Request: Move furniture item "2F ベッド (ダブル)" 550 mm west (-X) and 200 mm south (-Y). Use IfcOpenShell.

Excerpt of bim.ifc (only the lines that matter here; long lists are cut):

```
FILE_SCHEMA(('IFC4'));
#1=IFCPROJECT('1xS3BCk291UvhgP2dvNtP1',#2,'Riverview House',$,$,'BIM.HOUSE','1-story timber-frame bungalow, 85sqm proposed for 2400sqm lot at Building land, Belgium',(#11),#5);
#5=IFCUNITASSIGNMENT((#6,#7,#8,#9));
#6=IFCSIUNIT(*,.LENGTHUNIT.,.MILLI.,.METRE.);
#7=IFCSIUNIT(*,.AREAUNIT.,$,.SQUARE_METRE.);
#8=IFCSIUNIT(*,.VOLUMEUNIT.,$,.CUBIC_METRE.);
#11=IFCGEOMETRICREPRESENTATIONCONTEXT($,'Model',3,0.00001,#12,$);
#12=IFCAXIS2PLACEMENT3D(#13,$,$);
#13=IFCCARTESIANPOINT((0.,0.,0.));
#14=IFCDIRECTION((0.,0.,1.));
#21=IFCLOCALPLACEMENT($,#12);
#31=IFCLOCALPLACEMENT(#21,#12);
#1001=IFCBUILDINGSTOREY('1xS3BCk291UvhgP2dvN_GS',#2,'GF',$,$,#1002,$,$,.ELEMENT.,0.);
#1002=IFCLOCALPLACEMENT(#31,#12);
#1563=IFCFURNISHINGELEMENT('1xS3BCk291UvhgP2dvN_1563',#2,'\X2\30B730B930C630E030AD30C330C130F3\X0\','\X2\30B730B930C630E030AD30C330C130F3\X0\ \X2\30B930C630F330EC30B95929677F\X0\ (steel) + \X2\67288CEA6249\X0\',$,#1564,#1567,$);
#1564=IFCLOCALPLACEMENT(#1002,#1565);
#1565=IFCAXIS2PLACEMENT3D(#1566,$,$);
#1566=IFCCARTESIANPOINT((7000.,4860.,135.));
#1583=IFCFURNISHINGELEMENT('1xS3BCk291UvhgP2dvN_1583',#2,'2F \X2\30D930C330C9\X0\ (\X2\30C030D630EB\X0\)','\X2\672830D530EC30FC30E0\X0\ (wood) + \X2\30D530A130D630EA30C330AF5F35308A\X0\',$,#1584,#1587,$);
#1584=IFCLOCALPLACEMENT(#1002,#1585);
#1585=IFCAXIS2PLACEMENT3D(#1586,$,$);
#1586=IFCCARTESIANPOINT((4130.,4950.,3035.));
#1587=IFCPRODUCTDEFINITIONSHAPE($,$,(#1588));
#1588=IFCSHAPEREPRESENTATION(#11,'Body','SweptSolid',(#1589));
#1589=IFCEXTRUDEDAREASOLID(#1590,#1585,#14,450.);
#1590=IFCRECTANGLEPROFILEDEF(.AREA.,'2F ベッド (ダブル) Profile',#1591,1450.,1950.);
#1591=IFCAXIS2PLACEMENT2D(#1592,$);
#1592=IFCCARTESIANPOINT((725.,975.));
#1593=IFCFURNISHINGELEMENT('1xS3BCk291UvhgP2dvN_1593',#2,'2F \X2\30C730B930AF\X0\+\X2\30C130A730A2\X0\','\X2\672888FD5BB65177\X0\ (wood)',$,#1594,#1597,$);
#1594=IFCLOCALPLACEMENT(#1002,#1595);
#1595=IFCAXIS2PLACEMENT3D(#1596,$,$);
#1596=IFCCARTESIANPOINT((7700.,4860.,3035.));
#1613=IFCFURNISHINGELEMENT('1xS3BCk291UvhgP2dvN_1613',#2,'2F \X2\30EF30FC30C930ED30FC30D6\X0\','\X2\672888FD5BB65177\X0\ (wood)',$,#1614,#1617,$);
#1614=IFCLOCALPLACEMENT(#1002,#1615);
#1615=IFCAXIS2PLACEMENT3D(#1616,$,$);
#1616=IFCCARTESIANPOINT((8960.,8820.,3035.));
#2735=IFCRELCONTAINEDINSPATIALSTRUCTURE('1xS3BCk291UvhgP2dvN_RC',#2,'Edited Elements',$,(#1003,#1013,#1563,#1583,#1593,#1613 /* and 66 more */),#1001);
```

```python
import ifcopenshell
import ifcopenshell.api.geometry
import ifcopenshell.util.placement

model = ifcopenshell.open("bim.ifc")

item = model.by_guid("1xS3BCk291UvhgP2dvN_1583")
matrix = ifcopenshell.util.placement.get_local_placement(item.ObjectPlacement)
matrix[0, 3] -= 550.0
matrix[1, 3] -= 200.0
ifcopenshell.api.geometry.edit_object_placement(model, product=item, matrix=matrix, is_si=False)

print(ifcopenshell.util.placement.get_local_placement(item.ObjectPlacement).round(3) + 0.0)

model.write("bim_updated.ifc")
```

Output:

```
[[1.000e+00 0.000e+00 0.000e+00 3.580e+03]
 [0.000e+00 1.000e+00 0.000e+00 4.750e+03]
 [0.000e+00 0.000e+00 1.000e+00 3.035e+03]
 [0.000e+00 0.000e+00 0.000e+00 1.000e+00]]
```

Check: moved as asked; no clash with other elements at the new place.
